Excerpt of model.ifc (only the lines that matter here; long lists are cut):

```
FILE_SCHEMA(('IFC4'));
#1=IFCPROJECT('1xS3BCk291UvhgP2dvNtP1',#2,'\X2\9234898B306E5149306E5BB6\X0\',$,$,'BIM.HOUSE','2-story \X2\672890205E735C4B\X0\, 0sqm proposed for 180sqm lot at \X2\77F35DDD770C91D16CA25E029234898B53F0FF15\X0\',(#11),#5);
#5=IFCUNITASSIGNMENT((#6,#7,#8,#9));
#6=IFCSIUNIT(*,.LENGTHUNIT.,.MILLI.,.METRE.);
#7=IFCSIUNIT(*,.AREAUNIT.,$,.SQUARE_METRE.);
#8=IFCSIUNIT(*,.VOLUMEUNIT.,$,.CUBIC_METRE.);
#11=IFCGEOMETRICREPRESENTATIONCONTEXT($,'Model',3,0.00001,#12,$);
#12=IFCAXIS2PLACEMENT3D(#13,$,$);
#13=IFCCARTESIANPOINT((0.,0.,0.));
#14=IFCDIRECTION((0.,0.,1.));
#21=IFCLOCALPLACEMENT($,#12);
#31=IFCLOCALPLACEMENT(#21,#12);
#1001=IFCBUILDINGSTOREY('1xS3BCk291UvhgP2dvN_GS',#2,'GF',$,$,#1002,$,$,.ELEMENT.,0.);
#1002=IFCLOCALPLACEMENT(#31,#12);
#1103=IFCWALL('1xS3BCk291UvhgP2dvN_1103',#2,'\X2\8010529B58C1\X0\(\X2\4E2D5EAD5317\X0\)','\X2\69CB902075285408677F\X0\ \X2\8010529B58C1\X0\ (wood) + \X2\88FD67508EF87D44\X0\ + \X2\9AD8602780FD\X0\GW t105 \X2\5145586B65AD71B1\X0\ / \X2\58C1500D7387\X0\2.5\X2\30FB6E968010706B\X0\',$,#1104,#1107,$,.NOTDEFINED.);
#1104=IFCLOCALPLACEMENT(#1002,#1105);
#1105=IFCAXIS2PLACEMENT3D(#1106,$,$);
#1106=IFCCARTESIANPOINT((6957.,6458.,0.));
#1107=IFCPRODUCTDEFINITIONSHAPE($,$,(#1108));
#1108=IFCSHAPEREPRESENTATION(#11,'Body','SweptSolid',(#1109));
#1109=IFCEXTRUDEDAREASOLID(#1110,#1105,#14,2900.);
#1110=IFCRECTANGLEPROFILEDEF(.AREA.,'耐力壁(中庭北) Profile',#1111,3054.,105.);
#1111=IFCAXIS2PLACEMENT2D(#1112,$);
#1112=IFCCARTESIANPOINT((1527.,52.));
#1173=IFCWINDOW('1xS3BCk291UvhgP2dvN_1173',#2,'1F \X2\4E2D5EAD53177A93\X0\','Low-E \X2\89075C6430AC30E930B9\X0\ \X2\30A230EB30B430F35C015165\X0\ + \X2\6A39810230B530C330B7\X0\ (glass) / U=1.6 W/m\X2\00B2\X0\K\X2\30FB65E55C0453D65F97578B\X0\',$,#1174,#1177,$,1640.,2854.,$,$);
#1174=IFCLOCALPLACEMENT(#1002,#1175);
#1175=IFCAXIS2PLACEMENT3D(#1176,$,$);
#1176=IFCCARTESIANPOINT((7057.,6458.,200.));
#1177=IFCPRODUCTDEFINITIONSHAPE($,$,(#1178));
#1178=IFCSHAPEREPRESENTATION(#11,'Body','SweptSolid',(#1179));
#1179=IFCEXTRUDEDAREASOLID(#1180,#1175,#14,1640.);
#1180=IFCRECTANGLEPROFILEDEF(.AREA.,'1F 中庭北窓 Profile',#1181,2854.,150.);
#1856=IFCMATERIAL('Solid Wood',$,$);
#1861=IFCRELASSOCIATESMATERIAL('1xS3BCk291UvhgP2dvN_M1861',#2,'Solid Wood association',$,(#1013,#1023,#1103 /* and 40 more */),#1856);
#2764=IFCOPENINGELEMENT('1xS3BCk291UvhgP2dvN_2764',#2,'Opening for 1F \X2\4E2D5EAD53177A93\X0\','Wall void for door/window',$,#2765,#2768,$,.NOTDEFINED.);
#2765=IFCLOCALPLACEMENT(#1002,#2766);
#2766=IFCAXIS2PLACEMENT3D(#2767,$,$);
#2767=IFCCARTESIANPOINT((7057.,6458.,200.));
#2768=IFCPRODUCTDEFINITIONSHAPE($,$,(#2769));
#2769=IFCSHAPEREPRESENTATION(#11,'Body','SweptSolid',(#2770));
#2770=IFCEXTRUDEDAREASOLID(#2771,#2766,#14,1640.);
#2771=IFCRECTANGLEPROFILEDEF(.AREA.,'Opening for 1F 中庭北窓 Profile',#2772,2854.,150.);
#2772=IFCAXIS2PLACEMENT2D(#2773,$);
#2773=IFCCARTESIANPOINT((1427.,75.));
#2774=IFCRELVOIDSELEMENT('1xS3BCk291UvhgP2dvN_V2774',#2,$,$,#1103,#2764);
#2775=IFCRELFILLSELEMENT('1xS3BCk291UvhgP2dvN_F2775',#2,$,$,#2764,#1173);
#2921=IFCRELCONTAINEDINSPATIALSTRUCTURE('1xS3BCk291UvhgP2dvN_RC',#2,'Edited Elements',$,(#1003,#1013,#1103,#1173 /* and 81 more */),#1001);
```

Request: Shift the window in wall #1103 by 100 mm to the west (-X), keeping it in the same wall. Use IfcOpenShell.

```python
import ifcopenshell
import ifcopenshell.api.geometry
import ifcopenshell.util.placement
import ifcopenshell.util.unit

model = ifcopenshell.open("model.ifc")
unit_scale = ifcopenshell.util.unit.calculate_unit_scale(model)

window = model.by_id(1173)
opening = window.FillsVoids[0].RelatingOpeningElement
wall = opening.VoidsElements[0].RelatingBuildingElement

wall_matrix = ifcopenshell.util.placement.get_local_placement(wall.ObjectPlacement)
shift = wall_matrix[:3, 0] * -0.1 / unit_scale
before = ifcopenshell.util.placement.get_local_placement(window.ObjectPlacement)[:3, 3].copy()

# The window is not placed relative to its opening, so move both.
for product in (opening, window):
    matrix = ifcopenshell.util.placement.get_local_placement(product.ObjectPlacement)
    matrix[:3, 3] += shift
    ifcopenshell.api.geometry.edit_object_placement(model, product=product, matrix=matrix, is_si=False)

after = ifcopenshell.util.placement.get_local_placement(window.ObjectPlacement)[:3, 3]
print("window moved by", (after - before).round(3) + 0.0)

model.write("model_v2.ifc")
```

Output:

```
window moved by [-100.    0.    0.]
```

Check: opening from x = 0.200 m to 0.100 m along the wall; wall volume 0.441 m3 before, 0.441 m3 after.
